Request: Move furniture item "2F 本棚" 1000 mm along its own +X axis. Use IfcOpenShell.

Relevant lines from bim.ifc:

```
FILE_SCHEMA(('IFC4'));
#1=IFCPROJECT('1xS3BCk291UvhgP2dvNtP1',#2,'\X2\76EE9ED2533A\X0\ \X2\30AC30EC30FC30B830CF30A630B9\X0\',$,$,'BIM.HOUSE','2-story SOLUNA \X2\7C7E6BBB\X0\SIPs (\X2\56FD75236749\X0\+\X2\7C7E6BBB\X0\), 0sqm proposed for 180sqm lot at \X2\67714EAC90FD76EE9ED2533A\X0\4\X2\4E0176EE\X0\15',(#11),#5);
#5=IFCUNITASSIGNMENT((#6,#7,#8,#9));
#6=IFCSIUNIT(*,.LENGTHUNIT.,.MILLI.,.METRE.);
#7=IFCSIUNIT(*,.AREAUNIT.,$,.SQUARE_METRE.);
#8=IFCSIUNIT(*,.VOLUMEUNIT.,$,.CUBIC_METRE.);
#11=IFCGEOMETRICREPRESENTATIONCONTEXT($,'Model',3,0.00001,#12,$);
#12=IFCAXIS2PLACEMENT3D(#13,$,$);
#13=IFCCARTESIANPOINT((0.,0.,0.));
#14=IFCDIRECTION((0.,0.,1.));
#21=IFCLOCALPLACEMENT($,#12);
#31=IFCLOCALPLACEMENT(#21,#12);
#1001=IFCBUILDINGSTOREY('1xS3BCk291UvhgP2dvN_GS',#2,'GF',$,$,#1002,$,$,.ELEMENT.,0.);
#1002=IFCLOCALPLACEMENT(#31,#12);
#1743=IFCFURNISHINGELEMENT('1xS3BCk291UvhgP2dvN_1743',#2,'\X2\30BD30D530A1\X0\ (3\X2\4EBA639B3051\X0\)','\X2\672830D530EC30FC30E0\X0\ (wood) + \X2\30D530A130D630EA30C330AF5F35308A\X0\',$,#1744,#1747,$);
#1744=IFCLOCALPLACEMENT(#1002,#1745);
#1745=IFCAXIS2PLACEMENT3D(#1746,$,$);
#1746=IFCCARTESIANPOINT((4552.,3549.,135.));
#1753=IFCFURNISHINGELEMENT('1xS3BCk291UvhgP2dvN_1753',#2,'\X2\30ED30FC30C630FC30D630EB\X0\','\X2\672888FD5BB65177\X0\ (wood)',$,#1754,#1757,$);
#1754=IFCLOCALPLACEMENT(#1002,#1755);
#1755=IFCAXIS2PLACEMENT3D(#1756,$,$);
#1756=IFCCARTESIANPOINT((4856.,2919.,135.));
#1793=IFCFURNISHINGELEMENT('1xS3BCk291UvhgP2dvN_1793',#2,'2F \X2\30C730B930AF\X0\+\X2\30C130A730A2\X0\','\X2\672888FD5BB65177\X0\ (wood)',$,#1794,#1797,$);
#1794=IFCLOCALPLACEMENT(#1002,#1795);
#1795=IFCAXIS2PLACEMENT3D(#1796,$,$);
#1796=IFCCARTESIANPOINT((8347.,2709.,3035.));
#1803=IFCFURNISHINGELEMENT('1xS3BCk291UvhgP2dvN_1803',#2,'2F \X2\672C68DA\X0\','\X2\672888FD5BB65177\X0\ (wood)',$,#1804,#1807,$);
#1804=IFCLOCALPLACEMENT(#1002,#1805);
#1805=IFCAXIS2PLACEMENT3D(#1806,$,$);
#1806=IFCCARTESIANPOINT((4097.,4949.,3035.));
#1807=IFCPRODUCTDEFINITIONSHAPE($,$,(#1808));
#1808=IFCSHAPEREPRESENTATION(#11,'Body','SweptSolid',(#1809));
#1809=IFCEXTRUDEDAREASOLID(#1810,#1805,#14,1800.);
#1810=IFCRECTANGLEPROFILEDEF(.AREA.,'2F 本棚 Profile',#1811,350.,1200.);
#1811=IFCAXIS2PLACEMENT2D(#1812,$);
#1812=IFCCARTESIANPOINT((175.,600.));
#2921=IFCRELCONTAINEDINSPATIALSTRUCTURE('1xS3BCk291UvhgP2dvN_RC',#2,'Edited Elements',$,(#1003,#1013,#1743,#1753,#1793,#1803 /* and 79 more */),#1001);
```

```python
import ifcopenshell
import ifcopenshell.api.geometry
import ifcopenshell.util.placement

model = ifcopenshell.open("bim.ifc")

item = model.by_id(1803)
matrix = ifcopenshell.util.placement.get_local_placement(item.ObjectPlacement)
matrix[:3, 3] += matrix[:3, 0] * 1000.0
ifcopenshell.api.geometry.edit_object_placement(model, product=item, matrix=matrix, is_si=False)

print(ifcopenshell.util.placement.get_local_placement(item.ObjectPlacement).round(3) + 0.0)

model.write("bim_edited.ifc")
```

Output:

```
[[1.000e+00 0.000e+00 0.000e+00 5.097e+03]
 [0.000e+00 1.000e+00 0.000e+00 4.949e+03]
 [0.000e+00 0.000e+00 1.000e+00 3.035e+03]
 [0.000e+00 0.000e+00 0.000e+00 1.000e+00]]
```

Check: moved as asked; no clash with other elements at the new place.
